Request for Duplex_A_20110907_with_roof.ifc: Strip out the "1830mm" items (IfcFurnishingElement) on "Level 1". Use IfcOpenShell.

First a look at what the model holds.

```python
import ifcopenshell
import ifcopenshell.util.element

model = ifcopenshell.open("Duplex_A_20110907_with_roof.ifc")
print(model.schema)
storey = next(s for s in model.by_type("IfcBuildingStorey") if s.Name == "Level 1")
furniture = [e for e in ifcopenshell.util.element.get_decomposition(storey) if e.is_a("IfcFurnishingElement")]
seen = {}
for e in furniture:
    element_type = ifcopenshell.util.element.get_type(e)
    name = element_type.Name if element_type not in (None, e) else None
    seen[name] = seen.get(name, 0) + 1
for name, count in sorted(seen.items(), key=str):
    print(count, "x", name)
```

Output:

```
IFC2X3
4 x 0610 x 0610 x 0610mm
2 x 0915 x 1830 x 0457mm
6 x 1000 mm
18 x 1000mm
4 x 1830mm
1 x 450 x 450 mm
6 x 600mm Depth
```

```python
import ifcopenshell
import ifcopenshell.api.root
import ifcopenshell.util.element

model = ifcopenshell.open("Duplex_A_20110907_with_roof.ifc")

storey = next(s for s in model.by_type("IfcBuildingStorey") if s.Name == "Level 1")
furniture = [e for e in ifcopenshell.util.element.get_decomposition(storey) if e.is_a("IfcFurnishingElement")]
targets = [e for e in furniture if (t := ifcopenshell.util.element.get_type(e)) not in (None, e) and t.Name == "1830mm"]

for e in targets:
    ifcopenshell.api.root.remove_product(model, product=e)
print(len(targets), "removed")

model.write("Duplex_A_20110907_with_roof_updated.ifc")
```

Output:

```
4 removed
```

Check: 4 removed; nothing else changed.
